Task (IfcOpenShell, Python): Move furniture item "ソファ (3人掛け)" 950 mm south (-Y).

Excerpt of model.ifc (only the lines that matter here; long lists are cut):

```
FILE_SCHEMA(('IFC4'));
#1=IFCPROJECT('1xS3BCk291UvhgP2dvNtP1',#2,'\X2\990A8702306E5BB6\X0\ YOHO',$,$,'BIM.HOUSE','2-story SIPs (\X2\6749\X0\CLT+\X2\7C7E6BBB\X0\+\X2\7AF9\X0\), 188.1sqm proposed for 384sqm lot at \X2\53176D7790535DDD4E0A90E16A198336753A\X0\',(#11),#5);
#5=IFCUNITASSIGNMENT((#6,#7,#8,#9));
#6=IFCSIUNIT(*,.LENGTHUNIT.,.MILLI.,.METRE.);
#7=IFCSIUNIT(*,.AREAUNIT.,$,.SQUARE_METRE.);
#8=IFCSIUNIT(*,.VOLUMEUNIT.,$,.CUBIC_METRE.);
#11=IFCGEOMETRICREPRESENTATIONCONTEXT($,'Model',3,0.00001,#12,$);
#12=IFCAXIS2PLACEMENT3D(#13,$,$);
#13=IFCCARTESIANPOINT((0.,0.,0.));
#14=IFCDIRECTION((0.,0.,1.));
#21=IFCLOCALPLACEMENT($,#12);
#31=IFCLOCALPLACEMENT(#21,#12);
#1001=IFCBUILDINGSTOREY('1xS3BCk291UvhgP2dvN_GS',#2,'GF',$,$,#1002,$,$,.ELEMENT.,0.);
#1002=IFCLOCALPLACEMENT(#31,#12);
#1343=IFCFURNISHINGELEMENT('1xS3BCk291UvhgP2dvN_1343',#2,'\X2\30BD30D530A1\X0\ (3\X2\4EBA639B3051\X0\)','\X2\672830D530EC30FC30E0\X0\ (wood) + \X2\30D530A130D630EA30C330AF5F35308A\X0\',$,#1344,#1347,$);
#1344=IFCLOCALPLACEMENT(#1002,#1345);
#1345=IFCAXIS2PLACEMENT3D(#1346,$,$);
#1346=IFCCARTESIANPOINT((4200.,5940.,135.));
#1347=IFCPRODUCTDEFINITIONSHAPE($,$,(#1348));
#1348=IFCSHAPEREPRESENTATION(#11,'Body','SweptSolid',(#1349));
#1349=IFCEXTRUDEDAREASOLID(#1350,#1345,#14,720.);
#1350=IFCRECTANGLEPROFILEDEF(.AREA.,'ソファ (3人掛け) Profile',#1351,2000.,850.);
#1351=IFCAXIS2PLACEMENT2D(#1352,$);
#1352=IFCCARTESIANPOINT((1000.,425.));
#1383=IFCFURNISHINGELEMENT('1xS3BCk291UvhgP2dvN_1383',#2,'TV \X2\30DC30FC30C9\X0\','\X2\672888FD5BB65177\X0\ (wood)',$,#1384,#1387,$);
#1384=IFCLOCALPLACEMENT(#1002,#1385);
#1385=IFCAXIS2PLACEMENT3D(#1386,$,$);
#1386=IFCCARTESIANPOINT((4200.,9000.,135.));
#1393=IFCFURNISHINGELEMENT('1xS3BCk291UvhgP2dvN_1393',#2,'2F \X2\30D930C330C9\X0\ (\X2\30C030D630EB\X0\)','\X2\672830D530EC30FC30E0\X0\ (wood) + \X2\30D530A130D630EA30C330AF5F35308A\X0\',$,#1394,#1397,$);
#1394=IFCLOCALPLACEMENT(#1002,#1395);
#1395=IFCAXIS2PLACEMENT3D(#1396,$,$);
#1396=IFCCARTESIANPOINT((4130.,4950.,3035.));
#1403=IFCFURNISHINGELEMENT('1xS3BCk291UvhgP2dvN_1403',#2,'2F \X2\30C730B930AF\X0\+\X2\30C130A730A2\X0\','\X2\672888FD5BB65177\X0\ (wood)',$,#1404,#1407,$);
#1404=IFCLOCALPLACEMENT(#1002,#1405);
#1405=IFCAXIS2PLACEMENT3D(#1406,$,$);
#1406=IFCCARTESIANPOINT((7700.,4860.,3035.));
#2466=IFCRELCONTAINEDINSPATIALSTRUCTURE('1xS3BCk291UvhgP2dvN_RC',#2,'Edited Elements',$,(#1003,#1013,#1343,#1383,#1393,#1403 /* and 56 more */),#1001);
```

```python
import ifcopenshell
import ifcopenshell.api.geometry
import ifcopenshell.util.placement
import ifcopenshell.util.unit

model = ifcopenshell.open("model.ifc")
unit_scale = ifcopenshell.util.unit.calculate_unit_scale(model)

item = model.by_guid("1xS3BCk291UvhgP2dvN_1343")
matrix = ifcopenshell.util.placement.get_local_placement(item.ObjectPlacement)
matrix[1, 3] -= 0.95 / unit_scale
ifcopenshell.api.geometry.edit_object_placement(model, product=item, matrix=matrix, is_si=False)

print(ifcopenshell.util.placement.get_local_placement(item.ObjectPlacement).round(3) + 0.0)

model.write("model_v2.ifc")
```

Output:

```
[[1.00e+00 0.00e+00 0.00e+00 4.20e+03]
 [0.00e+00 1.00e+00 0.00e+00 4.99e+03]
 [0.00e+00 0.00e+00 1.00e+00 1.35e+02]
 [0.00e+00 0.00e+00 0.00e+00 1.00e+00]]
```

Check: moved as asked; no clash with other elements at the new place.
